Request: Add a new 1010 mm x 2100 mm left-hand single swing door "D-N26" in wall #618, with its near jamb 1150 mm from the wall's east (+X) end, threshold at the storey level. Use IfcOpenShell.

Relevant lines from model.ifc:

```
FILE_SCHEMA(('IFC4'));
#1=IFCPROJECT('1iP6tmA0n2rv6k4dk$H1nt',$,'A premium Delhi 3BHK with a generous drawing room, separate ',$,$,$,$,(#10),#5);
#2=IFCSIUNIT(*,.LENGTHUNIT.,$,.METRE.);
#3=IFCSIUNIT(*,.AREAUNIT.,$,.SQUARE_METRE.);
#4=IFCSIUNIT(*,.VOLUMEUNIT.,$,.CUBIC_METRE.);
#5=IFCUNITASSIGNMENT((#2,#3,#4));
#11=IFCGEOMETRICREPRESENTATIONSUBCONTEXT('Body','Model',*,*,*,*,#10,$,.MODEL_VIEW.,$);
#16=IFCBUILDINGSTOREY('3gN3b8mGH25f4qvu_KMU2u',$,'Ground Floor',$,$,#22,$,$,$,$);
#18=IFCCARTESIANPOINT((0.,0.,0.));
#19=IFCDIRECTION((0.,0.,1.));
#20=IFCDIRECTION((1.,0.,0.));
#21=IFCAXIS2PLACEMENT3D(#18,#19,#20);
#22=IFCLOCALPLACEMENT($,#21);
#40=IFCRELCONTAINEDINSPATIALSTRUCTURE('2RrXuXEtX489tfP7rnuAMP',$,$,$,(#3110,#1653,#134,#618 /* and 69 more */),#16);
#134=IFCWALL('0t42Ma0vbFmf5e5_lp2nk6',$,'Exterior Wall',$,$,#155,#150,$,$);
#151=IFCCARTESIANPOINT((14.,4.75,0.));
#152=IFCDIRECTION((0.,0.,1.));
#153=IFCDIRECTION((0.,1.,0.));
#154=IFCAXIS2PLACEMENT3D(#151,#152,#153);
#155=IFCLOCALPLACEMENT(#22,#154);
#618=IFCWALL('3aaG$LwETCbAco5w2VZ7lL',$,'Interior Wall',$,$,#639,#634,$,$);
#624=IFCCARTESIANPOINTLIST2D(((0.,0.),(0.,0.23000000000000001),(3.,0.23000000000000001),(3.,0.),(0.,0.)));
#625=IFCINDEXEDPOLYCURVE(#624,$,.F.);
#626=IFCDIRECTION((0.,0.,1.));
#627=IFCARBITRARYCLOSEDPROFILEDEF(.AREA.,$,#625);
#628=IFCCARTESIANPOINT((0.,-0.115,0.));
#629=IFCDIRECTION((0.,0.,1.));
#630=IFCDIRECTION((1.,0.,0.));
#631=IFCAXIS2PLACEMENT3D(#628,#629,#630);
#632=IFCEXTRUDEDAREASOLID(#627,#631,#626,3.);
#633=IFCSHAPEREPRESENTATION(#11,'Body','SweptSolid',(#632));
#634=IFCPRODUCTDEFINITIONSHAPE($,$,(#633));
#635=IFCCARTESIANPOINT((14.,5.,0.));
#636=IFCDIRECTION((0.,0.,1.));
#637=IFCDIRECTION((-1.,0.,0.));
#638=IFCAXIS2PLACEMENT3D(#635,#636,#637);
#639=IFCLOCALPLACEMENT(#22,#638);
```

```python
import numpy as np
import ifcopenshell
import ifcopenshell.api.feature
import ifcopenshell.api.geometry
import ifcopenshell.api.root
import ifcopenshell.api.spatial
import ifcopenshell.geom
import ifcopenshell.util.element
import ifcopenshell.util.placement
import ifcopenshell.util.representation
import ifcopenshell.util.shape
import ifcopenshell.util.unit

model = ifcopenshell.open("model.ifc")
unit_scale = ifcopenshell.util.unit.calculate_unit_scale(model)
settings = ifcopenshell.geom.settings()


def volume(element):
    """Net volume in cubic metres, openings subtracted."""
    shape = ifcopenshell.geom.create_shape(settings, element)
    return ifcopenshell.util.shape.get_volume(shape.geometry)


wall = model.by_id(618)
storey = ifcopenshell.util.element.get_container(wall, ifc_class="IfcBuildingStorey")
context = ifcopenshell.util.representation.get_context(model, "Model", "Body", "MODEL_VIEW")
before = volume(wall)

width, height, from_end, sill = 1.01, 2.1, 1.15, 0.0  # metres

# The wall runs along its own X axis, and the end named is its -X end.
wall_shape = ifcopenshell.geom.create_shape(settings, wall)
x, y, z = ifcopenshell.util.shape.get_vertices(wall_shape.geometry).T
start = x.min() + from_end
face, thickness = float(y.min()), float(y.max() - y.min())
wall_matrix = ifcopenshell.util.placement.get_local_placement(wall.ObjectPlacement)
level = ifcopenshell.util.placement.get_local_placement(storey.ObjectPlacement)[2, 3]


def in_wall(x, y):
    """Placement at x, y metres in the wall's axes, at sill height."""
    matrix = wall_matrix.copy()
    matrix[:, 3] = wall_matrix @ np.array([x / unit_scale, y / unit_scale, 0.0, 1.0])
    matrix[2, 3] = level + sill / unit_scale
    return matrix


# Opening: a box that overshoots both wall faces by 50 mm.
opening = ifcopenshell.api.root.create_entity(model, ifc_class="IfcOpeningElement", predefined_type="OPENING")
box = ifcopenshell.api.geometry.add_wall_representation(
    model, context=context, length=width, height=height, thickness=thickness + 0.1
)
ifcopenshell.api.geometry.assign_representation(model, product=opening, representation=box)
ifcopenshell.api.geometry.edit_object_placement(model, product=opening, matrix=in_wall(start, face - 0.05), is_si=False)
ifcopenshell.api.feature.add_feature(model, feature=opening, element=wall)

door = ifcopenshell.api.root.create_entity(model, ifc_class="IfcDoor", name="D-N26", predefined_type="DOOR")
door.OverallWidth, door.OverallHeight = width / unit_scale, height / unit_scale
door.OperationType = "SINGLE_SWING_LEFT"
body = ifcopenshell.api.geometry.add_door_representation(
    model,
    context=context,
    overall_width=door.OverallWidth,
    overall_height=door.OverallHeight,
    operation_type="SINGLE_SWING_LEFT",
    lining_properties={"LiningDepth": thickness / unit_scale, "ThresholdDepth": thickness / unit_scale},
)
ifcopenshell.api.geometry.assign_representation(model, product=door, representation=body)
ifcopenshell.api.spatial.assign_container(model, products=[door], relating_structure=storey)
ifcopenshell.api.feature.add_filling(model, opening=opening, element=door)

# The lining spans the wall, so the door starts at the wall face.
ifcopenshell.api.geometry.edit_object_placement(model, product=door, matrix=in_wall(start, face), is_si=False)

after = volume(wall)

print(f"wall volume {before:.3f} -> {after:.3f} m3")

model.write("model_rev.ifc")
```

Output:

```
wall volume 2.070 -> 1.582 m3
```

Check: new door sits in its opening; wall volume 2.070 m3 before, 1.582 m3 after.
